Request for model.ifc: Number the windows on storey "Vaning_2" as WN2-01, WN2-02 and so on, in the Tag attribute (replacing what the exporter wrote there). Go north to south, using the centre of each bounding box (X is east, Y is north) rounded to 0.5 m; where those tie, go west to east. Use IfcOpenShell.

First a look at what the model holds.

```python
import ifcopenshell
import ifcopenshell.util.element
import ifcopenshell.util.placement

model = ifcopenshell.open("model.ifc")
print(model.schema)
storey = next(s for s in model.by_type("IfcBuildingStorey") if s.Name == "Vaning_2")
windows = [e for e in ifcopenshell.util.element.get_decomposition(storey) if e.is_a("IfcWindow")]
for e in sorted(windows, key=lambda e: e.id()):
    origin = ifcopenshell.util.placement.get_local_placement(e.ObjectPlacement)[:3, 3]
    print(e.id(), e.Tag, e.Name, origin.round(2) + 0.0, sep=" | ")
```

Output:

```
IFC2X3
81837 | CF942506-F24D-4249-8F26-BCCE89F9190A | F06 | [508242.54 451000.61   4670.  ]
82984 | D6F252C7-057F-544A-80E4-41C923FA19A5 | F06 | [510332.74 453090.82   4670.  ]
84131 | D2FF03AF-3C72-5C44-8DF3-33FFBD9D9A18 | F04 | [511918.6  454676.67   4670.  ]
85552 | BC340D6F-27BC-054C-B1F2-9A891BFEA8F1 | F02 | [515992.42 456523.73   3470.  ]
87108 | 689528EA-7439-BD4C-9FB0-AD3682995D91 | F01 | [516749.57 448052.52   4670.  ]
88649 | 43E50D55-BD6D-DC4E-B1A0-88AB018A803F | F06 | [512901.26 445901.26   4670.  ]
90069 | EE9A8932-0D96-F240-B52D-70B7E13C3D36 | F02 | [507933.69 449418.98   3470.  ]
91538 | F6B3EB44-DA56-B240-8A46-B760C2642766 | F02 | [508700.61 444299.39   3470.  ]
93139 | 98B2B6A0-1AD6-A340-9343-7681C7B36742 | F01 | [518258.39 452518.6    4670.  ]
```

```python
import ifcopenshell
import ifcopenshell.geom
import ifcopenshell.util.element
import ifcopenshell.util.shape

model = ifcopenshell.open("model.ifc")
settings = ifcopenshell.geom.settings()
settings.set("use-world-coords", True)


def centre(element):
    shape = ifcopenshell.geom.create_shape(settings, element)
    return ifcopenshell.util.shape.get_bbox_centroid(shape.geometry)


storey = next(s for s in model.by_type("IfcBuildingStorey") if s.Name == "Vaning_2")
windows = [e for e in ifcopenshell.util.element.get_decomposition(storey) if e.is_a("IfcWindow")]

# Insertion points can sit at a corner or the storey origin, so sort by the geometry (in metres).
centres = {e: centre(e) for e in windows}
windows.sort(key=lambda e: (-round(centres[e][1] / 0.5), centres[e][0]))

for i, e in enumerate(windows, start=1):
    number = f"WN2-{i:02d}"
    e.Tag = number
    print(e.id(), number)

model.write("model_v2.ifc")
```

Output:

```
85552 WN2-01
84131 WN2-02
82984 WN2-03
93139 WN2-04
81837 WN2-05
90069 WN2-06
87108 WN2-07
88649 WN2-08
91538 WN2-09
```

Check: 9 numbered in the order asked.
